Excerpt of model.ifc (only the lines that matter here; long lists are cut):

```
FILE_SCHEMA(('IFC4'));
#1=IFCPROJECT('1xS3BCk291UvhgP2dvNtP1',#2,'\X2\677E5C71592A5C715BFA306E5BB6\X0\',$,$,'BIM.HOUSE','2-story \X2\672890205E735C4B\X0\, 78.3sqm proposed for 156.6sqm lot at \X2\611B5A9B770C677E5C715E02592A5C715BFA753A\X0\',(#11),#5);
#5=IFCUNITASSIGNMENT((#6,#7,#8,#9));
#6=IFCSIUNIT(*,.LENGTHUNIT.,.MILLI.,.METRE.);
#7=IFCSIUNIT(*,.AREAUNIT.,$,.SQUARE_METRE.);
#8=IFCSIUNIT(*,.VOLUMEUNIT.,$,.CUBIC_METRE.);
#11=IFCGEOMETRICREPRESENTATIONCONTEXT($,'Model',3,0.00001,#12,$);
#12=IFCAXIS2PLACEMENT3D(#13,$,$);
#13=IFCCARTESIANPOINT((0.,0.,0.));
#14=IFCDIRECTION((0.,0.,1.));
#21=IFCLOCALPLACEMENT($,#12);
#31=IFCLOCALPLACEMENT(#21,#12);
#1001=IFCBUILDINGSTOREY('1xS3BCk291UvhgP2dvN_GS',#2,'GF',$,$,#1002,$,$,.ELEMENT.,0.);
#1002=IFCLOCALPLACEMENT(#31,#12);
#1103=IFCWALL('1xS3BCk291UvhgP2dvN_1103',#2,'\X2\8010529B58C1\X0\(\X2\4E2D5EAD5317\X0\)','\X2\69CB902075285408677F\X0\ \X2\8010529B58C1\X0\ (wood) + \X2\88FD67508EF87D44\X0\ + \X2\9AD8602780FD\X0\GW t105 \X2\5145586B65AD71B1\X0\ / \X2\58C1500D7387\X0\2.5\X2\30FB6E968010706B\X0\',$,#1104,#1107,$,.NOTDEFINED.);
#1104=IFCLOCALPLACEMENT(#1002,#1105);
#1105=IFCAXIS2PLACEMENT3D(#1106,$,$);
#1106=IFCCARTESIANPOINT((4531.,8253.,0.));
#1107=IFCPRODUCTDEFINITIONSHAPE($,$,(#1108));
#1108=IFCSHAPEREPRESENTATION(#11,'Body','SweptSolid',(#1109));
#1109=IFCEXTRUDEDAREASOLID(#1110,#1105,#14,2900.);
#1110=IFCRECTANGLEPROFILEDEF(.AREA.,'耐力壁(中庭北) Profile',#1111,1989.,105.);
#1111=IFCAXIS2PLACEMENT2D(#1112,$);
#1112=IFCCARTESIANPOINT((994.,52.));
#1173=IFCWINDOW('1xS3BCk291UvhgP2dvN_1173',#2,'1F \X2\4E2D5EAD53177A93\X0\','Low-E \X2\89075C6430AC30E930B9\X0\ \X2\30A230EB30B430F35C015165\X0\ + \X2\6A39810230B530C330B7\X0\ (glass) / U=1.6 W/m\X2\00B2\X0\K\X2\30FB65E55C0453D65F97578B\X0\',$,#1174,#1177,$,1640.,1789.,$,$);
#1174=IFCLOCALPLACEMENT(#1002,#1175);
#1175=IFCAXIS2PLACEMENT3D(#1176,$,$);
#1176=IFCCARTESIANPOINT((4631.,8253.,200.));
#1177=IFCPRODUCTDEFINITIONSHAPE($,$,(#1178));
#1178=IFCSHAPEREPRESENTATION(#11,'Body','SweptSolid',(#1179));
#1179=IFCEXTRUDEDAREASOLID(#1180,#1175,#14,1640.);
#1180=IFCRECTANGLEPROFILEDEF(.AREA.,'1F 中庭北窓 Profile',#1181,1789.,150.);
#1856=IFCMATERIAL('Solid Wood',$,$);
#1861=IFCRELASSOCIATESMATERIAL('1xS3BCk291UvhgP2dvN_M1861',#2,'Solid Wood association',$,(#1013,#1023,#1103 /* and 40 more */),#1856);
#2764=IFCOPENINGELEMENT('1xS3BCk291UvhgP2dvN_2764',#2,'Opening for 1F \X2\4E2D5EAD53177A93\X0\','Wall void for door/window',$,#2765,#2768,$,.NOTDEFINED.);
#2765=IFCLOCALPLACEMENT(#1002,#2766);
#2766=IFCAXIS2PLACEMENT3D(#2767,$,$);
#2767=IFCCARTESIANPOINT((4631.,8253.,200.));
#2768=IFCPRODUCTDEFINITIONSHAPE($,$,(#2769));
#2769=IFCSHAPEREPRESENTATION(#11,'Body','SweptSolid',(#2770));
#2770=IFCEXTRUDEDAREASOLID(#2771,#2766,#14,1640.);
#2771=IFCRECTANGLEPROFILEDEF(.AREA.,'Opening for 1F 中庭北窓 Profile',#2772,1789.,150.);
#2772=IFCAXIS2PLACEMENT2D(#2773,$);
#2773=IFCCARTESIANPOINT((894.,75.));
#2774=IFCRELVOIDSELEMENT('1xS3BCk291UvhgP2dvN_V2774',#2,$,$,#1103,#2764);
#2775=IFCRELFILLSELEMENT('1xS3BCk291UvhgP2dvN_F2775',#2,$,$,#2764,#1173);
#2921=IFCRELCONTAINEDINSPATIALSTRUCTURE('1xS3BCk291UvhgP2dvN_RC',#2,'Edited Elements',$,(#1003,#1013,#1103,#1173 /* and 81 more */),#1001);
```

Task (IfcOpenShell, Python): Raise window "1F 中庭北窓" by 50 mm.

```python
import numpy as np
import ifcopenshell
import ifcopenshell.api.geometry
import ifcopenshell.util.placement
import ifcopenshell.util.unit

model = ifcopenshell.open("model.ifc")
unit_scale = ifcopenshell.util.unit.calculate_unit_scale(model)

window = model.by_guid("1xS3BCk291UvhgP2dvN_1173")
opening = window.FillsVoids[0].RelatingOpeningElement
dz = 0.05 / unit_scale

shift = np.array([0.0, 0.0, dz])
# The window is not placed relative to its opening, so move both.
for product in (opening, window):
    matrix = ifcopenshell.util.placement.get_local_placement(product.ObjectPlacement)
    matrix[:3, 3] += shift
    ifcopenshell.api.geometry.edit_object_placement(model, product=product, matrix=matrix, is_si=False)

print(f"moved by {dz * unit_scale:+.3f} m")

model.write("model_rev.ifc")
```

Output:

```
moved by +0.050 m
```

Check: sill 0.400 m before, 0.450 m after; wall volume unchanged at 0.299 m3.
